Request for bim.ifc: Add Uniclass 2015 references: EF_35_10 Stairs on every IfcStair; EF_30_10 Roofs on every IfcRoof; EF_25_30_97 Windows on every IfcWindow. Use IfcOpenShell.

First a look at what the model holds.

```python
import ifcopenshell

model = ifcopenshell.open("bim.ifc")
print(model.schema)
print("classifications:", [c.Name for c in model.by_type("IfcClassification")])
for ifc_class in ("IfcDoor", "IfcRoof", "IfcStair", "IfcWall", "IfcWindow"):
    print(ifc_class, len(model.by_type(ifc_class)))
```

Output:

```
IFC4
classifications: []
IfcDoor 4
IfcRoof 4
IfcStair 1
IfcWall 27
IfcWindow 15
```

```python
import ifcopenshell
import ifcopenshell.api.classification

model = ifcopenshell.open("bim.ifc")

system = ifcopenshell.api.classification.add_classification(model, classification="Uniclass 2015")

codes = {
    "IfcStair": ("EF_35_10", "Stairs"),
    "IfcRoof": ("EF_30_10", "Roofs"),
    "IfcWindow": ("EF_25_30_97", "Windows"),
}
for ifc_class, (code, name) in codes.items():
    products = model.by_type(ifc_class)
    ifcopenshell.api.classification.add_reference(
        model, products=products, classification=system, identification=code, name=name
    )
    print(code, len(products))

model.write("bim_edited.ifc")
```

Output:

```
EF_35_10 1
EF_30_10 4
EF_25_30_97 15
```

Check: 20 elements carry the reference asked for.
